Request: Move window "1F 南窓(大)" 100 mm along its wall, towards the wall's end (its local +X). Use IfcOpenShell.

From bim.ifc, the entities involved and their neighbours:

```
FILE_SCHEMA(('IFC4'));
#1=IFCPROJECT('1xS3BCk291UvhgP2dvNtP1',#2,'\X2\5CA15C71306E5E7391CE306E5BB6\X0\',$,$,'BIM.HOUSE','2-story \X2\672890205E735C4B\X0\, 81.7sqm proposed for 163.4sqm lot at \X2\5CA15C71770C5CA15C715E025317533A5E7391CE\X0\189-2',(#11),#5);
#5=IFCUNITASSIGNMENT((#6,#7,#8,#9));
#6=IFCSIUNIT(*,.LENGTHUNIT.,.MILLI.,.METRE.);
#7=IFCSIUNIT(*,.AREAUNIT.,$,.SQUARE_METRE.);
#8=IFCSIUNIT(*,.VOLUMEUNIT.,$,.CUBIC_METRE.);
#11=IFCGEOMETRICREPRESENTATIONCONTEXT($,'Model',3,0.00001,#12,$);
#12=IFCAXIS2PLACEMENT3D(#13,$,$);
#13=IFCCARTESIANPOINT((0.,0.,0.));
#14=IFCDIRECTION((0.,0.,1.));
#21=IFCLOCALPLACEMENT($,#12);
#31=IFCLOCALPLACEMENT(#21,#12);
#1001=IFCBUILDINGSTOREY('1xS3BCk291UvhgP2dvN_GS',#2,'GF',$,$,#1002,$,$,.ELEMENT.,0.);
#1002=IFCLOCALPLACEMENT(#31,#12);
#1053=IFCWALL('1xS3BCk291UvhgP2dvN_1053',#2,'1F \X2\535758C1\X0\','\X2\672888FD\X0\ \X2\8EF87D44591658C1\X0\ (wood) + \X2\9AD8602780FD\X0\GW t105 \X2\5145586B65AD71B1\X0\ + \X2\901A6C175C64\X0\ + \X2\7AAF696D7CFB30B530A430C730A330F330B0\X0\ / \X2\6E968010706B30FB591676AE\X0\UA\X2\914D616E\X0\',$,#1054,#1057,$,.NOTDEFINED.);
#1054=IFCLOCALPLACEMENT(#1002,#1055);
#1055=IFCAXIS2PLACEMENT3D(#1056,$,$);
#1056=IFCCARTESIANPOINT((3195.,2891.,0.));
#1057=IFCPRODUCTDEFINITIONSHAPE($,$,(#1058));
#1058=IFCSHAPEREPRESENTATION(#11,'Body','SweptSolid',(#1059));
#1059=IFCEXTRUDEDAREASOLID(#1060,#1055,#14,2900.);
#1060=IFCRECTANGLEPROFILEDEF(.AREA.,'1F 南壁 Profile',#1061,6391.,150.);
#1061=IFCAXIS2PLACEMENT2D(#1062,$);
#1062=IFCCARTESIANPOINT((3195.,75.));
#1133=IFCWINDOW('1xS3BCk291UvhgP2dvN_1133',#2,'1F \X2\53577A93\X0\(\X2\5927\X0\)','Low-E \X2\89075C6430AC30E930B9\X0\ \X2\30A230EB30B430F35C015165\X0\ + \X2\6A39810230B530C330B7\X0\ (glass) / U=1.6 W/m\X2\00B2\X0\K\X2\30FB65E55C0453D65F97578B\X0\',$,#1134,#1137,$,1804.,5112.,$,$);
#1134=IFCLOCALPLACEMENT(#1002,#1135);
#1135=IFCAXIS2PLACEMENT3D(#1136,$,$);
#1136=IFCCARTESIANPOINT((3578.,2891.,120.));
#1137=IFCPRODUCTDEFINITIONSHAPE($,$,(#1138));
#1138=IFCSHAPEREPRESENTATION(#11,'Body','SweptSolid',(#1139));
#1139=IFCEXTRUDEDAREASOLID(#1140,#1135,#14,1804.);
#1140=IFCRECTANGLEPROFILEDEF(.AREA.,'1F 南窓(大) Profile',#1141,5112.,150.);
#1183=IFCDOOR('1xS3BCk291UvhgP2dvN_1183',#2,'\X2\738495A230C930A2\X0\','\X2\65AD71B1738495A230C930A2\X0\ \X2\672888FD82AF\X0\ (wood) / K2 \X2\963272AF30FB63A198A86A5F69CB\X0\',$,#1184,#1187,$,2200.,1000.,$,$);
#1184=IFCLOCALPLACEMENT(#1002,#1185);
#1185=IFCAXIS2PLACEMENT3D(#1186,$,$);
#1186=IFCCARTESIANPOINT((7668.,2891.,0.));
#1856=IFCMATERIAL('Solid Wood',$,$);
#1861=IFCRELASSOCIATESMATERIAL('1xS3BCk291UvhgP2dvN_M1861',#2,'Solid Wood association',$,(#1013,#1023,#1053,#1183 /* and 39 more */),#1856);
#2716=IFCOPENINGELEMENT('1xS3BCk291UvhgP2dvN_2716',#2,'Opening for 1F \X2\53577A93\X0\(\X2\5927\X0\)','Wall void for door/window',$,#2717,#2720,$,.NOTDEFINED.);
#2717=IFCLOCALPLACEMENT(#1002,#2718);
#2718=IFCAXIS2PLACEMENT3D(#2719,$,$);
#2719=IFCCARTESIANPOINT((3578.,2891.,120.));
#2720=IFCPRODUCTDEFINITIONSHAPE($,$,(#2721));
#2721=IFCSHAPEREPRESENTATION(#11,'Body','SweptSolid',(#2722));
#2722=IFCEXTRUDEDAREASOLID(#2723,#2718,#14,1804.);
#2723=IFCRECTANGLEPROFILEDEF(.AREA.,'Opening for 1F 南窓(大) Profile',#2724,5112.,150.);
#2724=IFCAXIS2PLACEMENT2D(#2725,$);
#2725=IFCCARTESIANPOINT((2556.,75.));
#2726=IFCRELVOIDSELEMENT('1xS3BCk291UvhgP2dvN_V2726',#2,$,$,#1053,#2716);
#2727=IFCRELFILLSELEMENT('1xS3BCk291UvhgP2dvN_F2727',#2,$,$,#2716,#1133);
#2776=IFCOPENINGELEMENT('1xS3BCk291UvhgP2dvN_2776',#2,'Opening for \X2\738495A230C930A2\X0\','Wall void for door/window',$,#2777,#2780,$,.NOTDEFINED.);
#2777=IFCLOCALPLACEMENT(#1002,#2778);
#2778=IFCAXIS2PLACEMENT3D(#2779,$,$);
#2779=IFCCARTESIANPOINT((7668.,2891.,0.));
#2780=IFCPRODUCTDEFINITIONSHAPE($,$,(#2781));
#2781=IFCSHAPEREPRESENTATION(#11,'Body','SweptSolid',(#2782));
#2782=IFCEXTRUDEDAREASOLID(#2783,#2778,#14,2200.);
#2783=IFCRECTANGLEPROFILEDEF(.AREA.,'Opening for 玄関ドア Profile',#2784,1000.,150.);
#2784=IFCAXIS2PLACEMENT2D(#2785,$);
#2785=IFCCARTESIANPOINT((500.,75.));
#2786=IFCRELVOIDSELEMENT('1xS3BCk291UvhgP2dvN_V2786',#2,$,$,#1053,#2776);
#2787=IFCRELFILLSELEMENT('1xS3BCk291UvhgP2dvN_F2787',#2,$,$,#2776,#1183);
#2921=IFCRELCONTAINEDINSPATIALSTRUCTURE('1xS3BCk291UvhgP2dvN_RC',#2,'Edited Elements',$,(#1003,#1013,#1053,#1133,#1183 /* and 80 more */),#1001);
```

```python
import ifcopenshell
import ifcopenshell.api.geometry
import ifcopenshell.util.placement

model = ifcopenshell.open("bim.ifc")

window = model.by_guid("1xS3BCk291UvhgP2dvN_1133")
opening = window.FillsVoids[0].RelatingOpeningElement
wall = opening.VoidsElements[0].RelatingBuildingElement

wall_matrix = ifcopenshell.util.placement.get_local_placement(wall.ObjectPlacement)
shift = wall_matrix[:3, 0] * 100.0
before = ifcopenshell.util.placement.get_local_placement(window.ObjectPlacement)[:3, 3].copy()

# The window is not placed relative to its opening, so move both.
for product in (opening, window):
    matrix = ifcopenshell.util.placement.get_local_placement(product.ObjectPlacement)
    matrix[:3, 3] += shift
    ifcopenshell.api.geometry.edit_object_placement(model, product=product, matrix=matrix, is_si=False)

after = ifcopenshell.util.placement.get_local_placement(window.ObjectPlacement)[:3, 3]
print("window moved by", (after - before).round(3) + 0.0)

model.write("bim_rev.ifc")
```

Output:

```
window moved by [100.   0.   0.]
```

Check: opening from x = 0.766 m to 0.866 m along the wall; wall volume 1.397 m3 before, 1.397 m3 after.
